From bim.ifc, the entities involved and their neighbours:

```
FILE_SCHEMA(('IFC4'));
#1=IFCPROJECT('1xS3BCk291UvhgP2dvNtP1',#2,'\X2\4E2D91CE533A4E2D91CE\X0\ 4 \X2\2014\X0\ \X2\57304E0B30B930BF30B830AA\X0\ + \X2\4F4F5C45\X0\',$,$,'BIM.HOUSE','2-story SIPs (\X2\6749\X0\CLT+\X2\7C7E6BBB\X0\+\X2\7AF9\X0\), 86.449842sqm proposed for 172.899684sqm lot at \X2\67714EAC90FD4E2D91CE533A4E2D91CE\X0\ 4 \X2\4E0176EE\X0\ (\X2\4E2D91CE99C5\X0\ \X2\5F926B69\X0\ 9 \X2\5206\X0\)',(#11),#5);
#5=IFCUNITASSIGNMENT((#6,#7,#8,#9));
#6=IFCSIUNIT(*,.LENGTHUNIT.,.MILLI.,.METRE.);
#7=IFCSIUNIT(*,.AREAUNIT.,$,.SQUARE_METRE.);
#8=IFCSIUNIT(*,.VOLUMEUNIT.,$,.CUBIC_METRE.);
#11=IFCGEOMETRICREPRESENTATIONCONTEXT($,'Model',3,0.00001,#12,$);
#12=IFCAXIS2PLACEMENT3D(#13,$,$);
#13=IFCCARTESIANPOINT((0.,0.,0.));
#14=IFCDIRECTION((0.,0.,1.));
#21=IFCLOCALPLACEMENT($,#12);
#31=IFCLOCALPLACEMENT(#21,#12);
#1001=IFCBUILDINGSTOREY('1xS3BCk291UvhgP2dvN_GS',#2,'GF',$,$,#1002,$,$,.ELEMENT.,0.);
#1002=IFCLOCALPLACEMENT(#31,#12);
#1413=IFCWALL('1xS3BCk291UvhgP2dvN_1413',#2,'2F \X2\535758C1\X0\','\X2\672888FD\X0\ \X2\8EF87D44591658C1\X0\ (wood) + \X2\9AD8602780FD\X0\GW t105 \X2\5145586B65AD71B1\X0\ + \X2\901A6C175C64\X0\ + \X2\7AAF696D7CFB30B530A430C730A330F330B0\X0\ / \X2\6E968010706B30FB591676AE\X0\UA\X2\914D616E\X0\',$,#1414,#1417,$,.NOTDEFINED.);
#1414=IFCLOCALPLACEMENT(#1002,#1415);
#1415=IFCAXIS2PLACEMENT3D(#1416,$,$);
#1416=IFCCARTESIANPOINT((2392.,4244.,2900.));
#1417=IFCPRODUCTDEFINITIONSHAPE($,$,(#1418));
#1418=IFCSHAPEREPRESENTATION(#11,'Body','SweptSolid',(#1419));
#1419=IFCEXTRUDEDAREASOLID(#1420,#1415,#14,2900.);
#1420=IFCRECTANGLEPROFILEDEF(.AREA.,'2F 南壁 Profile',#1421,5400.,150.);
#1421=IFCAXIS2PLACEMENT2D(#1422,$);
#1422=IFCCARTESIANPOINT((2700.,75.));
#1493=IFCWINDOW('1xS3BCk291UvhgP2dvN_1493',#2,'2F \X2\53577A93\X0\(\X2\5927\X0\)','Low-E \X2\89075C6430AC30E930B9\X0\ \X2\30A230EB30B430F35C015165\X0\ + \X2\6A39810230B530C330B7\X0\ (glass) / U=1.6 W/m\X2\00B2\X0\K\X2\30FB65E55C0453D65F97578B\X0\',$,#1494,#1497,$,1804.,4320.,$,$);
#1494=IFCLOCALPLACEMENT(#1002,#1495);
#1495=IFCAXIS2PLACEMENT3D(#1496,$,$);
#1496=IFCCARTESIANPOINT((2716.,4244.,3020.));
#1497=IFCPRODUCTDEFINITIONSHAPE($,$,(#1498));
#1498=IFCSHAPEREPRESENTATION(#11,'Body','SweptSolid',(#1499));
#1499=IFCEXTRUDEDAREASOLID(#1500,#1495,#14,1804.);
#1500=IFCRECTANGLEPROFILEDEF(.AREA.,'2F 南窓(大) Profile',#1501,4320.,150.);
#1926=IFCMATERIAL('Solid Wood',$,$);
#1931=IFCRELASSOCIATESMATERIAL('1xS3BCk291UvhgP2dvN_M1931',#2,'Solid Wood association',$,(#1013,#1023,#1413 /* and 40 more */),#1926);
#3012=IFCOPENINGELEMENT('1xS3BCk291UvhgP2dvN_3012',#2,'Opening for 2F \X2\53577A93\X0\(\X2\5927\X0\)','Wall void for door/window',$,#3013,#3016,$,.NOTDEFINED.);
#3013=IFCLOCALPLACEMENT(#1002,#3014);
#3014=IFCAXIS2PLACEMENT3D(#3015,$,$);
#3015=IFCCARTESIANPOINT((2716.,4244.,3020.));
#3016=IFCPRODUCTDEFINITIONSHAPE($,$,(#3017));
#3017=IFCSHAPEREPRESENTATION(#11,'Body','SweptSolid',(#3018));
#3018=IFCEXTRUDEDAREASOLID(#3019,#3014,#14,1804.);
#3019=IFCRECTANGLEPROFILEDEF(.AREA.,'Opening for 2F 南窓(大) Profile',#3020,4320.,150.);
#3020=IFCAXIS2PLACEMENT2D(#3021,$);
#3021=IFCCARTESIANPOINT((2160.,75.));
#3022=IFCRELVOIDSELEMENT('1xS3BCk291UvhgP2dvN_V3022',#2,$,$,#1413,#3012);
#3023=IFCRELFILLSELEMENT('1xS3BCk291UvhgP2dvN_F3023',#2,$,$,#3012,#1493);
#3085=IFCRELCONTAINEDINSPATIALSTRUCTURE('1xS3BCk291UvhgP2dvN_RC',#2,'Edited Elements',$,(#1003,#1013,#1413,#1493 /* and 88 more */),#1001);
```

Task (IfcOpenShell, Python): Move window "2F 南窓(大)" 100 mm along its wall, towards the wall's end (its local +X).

```python
import ifcopenshell
import ifcopenshell.api.geometry
import ifcopenshell.util.placement
import ifcopenshell.util.unit

model = ifcopenshell.open("bim.ifc")
unit_scale = ifcopenshell.util.unit.calculate_unit_scale(model)

window = model.by_id(1493)
opening = window.FillsVoids[0].RelatingOpeningElement
wall = opening.VoidsElements[0].RelatingBuildingElement

wall_matrix = ifcopenshell.util.placement.get_local_placement(wall.ObjectPlacement)
shift = wall_matrix[:3, 0] * 0.1 / unit_scale
before = ifcopenshell.util.placement.get_local_placement(window.ObjectPlacement)[:3, 3].copy()

# The window is not placed relative to its opening, so move both.
for product in (opening, window):
    matrix = ifcopenshell.util.placement.get_local_placement(product.ObjectPlacement)
    matrix[:3, 3] += shift
    ifcopenshell.api.geometry.edit_object_placement(model, product=product, matrix=matrix, is_si=False)

after = ifcopenshell.util.placement.get_local_placement(window.ObjectPlacement)[:3, 3]
print("window moved by", (after - before).round(3) + 0.0)

model.write("bim_v2.ifc")
```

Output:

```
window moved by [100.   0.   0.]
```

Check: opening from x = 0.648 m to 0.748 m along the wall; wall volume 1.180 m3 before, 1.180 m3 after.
